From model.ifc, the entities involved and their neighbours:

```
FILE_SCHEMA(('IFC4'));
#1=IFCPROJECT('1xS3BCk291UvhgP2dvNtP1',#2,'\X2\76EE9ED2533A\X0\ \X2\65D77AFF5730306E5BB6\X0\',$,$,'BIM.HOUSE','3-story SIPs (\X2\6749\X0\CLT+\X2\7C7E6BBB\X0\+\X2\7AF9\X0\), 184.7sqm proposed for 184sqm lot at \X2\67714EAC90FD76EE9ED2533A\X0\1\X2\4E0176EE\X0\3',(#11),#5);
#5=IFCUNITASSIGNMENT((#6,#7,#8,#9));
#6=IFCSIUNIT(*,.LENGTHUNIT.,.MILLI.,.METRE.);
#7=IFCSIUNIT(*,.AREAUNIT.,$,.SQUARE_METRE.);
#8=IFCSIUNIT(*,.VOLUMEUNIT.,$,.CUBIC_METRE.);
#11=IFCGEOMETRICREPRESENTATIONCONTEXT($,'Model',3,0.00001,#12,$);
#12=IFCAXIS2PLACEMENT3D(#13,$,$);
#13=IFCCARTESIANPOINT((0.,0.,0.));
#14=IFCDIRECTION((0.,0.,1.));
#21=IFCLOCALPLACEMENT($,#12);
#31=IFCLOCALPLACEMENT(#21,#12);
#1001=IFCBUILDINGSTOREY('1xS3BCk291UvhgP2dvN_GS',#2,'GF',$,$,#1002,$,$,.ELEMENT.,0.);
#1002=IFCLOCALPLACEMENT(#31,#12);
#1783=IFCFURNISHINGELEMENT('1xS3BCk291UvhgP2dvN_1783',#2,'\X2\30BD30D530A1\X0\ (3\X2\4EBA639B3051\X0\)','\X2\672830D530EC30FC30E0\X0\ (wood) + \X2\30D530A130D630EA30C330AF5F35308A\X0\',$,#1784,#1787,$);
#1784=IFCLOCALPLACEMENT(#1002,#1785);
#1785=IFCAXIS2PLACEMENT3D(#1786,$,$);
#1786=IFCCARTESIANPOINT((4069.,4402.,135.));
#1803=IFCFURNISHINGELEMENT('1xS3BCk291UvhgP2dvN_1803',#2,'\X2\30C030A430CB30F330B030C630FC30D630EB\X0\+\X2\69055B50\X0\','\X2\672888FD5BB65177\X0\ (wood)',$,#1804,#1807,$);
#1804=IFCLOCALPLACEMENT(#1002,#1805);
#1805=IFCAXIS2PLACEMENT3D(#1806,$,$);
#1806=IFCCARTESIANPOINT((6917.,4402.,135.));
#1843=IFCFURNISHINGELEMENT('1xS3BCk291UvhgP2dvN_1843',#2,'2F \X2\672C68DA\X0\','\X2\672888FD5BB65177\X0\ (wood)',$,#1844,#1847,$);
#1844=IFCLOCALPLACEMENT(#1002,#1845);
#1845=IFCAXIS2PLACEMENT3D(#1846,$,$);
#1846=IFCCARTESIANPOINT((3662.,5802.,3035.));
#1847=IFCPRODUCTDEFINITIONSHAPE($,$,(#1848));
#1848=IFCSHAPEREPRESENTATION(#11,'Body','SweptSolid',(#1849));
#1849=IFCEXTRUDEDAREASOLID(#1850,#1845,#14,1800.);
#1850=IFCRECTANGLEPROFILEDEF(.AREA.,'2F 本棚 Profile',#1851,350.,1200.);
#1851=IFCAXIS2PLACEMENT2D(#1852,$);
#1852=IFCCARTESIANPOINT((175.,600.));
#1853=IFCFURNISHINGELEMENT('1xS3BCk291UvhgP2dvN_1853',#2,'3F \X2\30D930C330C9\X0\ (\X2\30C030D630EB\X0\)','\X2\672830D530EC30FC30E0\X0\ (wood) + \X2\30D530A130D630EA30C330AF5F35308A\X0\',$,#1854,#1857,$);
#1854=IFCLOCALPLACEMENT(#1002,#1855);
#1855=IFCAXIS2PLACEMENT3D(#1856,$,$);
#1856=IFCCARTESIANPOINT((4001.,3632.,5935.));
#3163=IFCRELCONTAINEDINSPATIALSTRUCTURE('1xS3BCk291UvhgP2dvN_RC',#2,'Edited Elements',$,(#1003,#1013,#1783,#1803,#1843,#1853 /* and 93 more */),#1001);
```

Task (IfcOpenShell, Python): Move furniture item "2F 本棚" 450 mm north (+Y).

```python
import ifcopenshell
import ifcopenshell.api.geometry
import ifcopenshell.util.placement
import ifcopenshell.util.unit

model = ifcopenshell.open("model.ifc")
unit_scale = ifcopenshell.util.unit.calculate_unit_scale(model)

item = model.by_guid("1xS3BCk291UvhgP2dvN_1843")
matrix = ifcopenshell.util.placement.get_local_placement(item.ObjectPlacement)
matrix[1, 3] += 0.45 / unit_scale
ifcopenshell.api.geometry.edit_object_placement(model, product=item, matrix=matrix, is_si=False)

print(ifcopenshell.util.placement.get_local_placement(item.ObjectPlacement).round(3) + 0.0)

model.write("model_v2.ifc")
```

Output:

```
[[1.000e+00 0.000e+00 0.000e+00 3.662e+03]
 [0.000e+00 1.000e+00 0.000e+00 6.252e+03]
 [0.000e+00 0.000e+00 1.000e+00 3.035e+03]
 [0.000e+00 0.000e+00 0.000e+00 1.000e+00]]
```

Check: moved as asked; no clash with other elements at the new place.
